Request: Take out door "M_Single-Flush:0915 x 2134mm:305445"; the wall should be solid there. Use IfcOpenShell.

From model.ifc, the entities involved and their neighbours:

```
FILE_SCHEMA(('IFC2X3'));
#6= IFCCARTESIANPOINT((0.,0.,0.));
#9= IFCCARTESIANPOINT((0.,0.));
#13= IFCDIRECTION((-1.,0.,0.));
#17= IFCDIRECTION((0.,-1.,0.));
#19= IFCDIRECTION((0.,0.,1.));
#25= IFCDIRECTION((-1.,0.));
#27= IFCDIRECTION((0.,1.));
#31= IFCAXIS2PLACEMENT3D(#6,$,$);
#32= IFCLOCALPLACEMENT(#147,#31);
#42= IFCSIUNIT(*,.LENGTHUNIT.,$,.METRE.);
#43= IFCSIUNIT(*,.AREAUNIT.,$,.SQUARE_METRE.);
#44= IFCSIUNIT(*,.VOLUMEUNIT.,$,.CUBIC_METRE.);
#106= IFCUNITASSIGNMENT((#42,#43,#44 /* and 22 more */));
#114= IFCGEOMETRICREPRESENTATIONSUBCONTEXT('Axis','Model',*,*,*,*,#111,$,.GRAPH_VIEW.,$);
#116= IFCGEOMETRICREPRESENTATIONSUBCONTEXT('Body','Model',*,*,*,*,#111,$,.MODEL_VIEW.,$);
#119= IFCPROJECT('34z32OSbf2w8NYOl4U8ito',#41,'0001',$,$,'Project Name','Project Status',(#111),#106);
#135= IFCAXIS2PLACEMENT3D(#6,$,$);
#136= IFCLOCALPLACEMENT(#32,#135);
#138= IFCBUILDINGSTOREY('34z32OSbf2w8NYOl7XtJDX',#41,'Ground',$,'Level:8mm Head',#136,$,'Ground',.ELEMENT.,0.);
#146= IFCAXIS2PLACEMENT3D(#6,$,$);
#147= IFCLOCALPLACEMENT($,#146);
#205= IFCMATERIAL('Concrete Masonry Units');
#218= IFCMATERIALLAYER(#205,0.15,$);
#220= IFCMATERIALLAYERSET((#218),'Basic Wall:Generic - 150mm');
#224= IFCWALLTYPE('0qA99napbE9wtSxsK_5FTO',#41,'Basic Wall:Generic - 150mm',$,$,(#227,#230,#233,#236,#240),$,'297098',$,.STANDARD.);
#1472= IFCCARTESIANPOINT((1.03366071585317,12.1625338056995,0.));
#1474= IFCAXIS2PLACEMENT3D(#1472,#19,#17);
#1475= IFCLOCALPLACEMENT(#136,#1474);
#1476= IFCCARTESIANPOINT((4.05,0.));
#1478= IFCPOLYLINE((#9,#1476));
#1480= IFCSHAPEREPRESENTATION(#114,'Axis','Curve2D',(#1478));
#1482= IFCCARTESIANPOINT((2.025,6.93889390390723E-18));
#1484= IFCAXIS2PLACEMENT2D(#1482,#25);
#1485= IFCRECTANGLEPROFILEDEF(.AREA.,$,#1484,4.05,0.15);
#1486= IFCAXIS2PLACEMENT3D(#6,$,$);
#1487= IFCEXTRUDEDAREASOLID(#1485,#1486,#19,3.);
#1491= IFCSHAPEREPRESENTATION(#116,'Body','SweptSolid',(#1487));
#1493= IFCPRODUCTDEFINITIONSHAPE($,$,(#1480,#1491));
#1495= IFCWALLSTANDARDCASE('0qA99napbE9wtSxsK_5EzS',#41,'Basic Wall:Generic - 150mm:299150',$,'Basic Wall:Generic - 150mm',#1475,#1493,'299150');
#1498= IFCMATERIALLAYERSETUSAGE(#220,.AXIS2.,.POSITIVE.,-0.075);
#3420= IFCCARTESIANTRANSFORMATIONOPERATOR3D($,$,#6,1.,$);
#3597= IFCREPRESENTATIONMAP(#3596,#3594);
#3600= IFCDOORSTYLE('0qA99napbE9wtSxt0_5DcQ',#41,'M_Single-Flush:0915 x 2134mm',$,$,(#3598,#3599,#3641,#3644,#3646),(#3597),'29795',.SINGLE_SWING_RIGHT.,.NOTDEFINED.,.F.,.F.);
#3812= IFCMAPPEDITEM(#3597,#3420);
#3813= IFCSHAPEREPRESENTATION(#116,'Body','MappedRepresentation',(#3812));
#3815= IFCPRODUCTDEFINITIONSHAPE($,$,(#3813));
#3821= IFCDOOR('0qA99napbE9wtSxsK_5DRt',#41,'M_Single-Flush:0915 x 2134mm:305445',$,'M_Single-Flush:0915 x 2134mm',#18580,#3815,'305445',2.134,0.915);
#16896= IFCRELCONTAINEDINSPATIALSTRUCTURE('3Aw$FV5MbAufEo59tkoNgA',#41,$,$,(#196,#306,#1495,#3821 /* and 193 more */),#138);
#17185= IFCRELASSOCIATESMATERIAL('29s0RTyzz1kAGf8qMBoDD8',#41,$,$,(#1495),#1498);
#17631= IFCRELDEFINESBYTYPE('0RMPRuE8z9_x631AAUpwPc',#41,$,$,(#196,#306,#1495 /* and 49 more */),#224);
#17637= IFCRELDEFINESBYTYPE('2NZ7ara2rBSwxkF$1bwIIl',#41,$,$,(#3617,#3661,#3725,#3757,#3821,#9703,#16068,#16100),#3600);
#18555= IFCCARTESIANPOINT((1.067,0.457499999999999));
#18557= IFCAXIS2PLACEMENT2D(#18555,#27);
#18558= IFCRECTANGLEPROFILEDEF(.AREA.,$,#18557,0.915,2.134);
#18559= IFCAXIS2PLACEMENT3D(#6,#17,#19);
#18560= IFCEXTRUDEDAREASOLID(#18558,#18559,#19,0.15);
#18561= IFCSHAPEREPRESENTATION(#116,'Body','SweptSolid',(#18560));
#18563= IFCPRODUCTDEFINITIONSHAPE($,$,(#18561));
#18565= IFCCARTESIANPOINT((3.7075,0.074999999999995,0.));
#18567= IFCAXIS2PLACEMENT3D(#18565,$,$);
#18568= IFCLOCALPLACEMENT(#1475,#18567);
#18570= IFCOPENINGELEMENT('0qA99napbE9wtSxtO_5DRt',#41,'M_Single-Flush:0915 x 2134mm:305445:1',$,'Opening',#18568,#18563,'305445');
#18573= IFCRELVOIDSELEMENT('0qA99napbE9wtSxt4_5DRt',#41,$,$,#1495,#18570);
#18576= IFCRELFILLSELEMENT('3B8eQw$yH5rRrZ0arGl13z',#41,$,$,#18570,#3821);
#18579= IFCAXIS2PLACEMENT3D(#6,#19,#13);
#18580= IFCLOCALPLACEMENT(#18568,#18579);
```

```python
import ifcopenshell
import ifcopenshell.api.feature
import ifcopenshell.api.root
import ifcopenshell.geom
import ifcopenshell.util.shape

model = ifcopenshell.open("model.ifc")
settings = ifcopenshell.geom.settings()


def volume(element):
    """Net volume in cubic metres, openings subtracted."""
    shape = ifcopenshell.geom.create_shape(settings, element)
    return ifcopenshell.util.shape.get_volume(shape.geometry)


door = model.by_guid("0qA99napbE9wtSxsK_5DRt")
opening = door.FillsVoids[0].RelatingOpeningElement
wall = opening.VoidsElements[0].RelatingBuildingElement
before = volume(wall)

ifcopenshell.api.root.remove_product(model, product=door)
ifcopenshell.api.feature.remove_feature(model, feature=opening)

after = volume(wall)

print(f"wall volume {before:.3f} -> {after:.3f} m3")

model.write("model_rev.ifc")
```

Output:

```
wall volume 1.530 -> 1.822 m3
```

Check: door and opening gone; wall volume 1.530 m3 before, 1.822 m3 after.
